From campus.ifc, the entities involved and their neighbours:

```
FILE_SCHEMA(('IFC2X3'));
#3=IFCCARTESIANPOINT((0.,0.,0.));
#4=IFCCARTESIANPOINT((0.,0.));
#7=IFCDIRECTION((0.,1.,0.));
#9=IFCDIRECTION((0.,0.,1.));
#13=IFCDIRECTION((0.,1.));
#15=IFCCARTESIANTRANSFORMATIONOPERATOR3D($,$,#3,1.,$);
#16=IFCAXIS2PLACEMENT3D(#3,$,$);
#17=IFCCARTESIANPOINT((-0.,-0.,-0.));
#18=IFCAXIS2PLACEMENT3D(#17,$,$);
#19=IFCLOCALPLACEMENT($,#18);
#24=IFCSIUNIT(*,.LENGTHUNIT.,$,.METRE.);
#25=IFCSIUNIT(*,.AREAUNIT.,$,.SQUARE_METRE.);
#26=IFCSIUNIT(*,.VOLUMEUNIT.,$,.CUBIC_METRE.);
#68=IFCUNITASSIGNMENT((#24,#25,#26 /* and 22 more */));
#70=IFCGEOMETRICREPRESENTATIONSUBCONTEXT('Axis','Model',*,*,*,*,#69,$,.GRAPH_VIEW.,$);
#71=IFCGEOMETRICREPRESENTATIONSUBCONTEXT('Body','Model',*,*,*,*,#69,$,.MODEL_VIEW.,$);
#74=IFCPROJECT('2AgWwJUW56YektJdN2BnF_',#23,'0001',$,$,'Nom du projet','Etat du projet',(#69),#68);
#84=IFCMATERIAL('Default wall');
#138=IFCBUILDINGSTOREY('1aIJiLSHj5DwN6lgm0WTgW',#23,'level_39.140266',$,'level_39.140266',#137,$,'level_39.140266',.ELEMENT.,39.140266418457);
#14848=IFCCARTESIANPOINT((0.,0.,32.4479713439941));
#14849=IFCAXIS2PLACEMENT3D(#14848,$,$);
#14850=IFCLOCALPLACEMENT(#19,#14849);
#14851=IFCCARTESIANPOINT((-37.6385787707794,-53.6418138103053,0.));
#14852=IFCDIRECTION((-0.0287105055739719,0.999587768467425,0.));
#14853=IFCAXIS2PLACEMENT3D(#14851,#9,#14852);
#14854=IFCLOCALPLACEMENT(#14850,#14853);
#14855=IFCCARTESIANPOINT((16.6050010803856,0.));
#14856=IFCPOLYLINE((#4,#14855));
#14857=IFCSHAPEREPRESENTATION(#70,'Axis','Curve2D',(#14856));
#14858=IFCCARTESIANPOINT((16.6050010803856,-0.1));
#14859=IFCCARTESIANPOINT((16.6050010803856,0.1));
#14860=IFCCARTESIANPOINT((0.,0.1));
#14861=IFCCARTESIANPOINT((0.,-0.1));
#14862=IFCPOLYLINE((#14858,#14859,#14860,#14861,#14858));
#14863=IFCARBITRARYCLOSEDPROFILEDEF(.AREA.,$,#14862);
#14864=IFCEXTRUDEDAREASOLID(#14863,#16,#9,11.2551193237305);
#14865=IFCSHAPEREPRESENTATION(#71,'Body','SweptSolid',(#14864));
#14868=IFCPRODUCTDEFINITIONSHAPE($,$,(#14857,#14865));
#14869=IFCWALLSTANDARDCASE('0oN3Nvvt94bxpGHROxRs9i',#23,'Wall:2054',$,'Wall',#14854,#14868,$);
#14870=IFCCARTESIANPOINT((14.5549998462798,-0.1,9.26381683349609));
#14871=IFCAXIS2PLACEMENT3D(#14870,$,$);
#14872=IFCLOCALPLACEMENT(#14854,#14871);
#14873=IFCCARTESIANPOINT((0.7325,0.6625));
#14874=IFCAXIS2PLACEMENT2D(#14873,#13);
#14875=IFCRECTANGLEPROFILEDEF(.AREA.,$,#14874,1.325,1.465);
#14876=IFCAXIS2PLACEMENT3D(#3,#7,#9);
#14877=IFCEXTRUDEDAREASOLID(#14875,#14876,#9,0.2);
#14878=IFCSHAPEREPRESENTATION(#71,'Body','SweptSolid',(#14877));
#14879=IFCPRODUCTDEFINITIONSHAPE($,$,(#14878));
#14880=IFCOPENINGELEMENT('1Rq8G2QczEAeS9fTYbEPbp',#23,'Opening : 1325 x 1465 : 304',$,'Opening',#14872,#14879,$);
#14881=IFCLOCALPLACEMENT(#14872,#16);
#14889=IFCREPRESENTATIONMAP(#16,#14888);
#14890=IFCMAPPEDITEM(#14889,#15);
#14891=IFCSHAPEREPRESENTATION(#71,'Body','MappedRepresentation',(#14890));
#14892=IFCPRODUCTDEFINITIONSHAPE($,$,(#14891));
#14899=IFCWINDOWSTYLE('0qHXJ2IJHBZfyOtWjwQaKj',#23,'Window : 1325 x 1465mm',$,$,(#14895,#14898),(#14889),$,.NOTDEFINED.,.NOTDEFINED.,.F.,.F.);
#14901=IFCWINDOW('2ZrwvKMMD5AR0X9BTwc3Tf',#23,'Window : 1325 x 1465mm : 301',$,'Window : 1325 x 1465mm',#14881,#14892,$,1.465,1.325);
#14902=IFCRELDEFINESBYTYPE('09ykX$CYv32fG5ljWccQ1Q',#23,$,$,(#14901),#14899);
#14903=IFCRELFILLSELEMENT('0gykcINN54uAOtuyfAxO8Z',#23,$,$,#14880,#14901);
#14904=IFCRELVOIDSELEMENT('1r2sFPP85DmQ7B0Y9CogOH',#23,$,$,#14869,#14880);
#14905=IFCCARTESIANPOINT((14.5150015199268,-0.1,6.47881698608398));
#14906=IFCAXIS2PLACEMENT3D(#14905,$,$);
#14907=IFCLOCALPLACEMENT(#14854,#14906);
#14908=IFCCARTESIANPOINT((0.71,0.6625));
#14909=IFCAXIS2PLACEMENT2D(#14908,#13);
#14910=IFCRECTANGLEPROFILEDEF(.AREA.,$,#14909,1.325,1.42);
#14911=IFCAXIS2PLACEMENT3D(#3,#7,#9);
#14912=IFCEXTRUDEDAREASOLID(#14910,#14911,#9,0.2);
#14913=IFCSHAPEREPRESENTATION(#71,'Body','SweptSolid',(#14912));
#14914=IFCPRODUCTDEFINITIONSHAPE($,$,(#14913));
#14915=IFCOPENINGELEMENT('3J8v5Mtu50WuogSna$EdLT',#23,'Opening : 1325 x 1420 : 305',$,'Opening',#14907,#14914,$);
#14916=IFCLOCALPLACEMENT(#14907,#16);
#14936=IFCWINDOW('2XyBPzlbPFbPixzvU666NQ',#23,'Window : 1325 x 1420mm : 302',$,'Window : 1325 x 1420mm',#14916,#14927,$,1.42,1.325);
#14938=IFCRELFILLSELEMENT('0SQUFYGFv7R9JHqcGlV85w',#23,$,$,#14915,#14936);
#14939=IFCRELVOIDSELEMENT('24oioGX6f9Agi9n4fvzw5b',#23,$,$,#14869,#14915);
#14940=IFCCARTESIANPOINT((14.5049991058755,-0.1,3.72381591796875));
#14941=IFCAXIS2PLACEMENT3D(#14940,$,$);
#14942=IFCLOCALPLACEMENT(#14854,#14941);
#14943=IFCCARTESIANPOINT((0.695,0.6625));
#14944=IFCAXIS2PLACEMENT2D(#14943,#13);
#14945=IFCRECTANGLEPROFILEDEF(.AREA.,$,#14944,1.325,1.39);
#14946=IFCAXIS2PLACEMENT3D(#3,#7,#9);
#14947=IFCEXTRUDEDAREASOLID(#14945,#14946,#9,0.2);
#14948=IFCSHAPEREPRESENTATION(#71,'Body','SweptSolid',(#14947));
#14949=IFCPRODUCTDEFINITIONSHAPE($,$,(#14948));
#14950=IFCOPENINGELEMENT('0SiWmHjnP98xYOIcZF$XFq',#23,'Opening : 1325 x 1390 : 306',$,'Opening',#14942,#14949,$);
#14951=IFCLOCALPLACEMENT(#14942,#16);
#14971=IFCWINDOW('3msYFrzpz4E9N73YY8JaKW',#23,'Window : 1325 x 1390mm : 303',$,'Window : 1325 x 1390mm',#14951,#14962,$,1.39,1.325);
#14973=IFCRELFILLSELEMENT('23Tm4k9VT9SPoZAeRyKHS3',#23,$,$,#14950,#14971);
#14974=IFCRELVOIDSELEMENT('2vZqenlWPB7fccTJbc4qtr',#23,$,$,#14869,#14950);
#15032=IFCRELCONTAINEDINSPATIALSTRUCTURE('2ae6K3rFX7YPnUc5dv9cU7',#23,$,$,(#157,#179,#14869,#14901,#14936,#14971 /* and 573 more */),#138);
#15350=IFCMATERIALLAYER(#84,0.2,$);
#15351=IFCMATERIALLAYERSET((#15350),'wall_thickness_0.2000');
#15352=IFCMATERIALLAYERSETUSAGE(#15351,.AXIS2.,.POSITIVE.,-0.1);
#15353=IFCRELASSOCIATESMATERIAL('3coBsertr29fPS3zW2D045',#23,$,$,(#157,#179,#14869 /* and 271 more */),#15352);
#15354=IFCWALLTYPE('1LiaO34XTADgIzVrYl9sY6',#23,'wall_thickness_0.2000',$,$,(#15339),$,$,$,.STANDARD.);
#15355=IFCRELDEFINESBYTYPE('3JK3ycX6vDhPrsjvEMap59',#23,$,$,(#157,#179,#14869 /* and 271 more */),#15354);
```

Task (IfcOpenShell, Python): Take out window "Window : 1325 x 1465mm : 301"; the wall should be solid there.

```python
import ifcopenshell
import ifcopenshell.api.feature
import ifcopenshell.api.root
import ifcopenshell.geom
import ifcopenshell.util.shape

model = ifcopenshell.open("campus.ifc")
settings = ifcopenshell.geom.settings()


def volume(element):
    """Net volume in cubic metres, openings subtracted."""
    shape = ifcopenshell.geom.create_shape(settings, element)
    return ifcopenshell.util.shape.get_volume(shape.geometry)


window = model.by_id(14901)
opening = window.FillsVoids[0].RelatingOpeningElement
wall = opening.VoidsElements[0].RelatingBuildingElement
before = volume(wall)

ifcopenshell.api.root.remove_product(model, product=window)
ifcopenshell.api.feature.remove_feature(model, feature=opening)

after = volume(wall)

print(f"wall volume {before:.3f} -> {after:.3f} m3")

model.write("campus_rev.ifc")
```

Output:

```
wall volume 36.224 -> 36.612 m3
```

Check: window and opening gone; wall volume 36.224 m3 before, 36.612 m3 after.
